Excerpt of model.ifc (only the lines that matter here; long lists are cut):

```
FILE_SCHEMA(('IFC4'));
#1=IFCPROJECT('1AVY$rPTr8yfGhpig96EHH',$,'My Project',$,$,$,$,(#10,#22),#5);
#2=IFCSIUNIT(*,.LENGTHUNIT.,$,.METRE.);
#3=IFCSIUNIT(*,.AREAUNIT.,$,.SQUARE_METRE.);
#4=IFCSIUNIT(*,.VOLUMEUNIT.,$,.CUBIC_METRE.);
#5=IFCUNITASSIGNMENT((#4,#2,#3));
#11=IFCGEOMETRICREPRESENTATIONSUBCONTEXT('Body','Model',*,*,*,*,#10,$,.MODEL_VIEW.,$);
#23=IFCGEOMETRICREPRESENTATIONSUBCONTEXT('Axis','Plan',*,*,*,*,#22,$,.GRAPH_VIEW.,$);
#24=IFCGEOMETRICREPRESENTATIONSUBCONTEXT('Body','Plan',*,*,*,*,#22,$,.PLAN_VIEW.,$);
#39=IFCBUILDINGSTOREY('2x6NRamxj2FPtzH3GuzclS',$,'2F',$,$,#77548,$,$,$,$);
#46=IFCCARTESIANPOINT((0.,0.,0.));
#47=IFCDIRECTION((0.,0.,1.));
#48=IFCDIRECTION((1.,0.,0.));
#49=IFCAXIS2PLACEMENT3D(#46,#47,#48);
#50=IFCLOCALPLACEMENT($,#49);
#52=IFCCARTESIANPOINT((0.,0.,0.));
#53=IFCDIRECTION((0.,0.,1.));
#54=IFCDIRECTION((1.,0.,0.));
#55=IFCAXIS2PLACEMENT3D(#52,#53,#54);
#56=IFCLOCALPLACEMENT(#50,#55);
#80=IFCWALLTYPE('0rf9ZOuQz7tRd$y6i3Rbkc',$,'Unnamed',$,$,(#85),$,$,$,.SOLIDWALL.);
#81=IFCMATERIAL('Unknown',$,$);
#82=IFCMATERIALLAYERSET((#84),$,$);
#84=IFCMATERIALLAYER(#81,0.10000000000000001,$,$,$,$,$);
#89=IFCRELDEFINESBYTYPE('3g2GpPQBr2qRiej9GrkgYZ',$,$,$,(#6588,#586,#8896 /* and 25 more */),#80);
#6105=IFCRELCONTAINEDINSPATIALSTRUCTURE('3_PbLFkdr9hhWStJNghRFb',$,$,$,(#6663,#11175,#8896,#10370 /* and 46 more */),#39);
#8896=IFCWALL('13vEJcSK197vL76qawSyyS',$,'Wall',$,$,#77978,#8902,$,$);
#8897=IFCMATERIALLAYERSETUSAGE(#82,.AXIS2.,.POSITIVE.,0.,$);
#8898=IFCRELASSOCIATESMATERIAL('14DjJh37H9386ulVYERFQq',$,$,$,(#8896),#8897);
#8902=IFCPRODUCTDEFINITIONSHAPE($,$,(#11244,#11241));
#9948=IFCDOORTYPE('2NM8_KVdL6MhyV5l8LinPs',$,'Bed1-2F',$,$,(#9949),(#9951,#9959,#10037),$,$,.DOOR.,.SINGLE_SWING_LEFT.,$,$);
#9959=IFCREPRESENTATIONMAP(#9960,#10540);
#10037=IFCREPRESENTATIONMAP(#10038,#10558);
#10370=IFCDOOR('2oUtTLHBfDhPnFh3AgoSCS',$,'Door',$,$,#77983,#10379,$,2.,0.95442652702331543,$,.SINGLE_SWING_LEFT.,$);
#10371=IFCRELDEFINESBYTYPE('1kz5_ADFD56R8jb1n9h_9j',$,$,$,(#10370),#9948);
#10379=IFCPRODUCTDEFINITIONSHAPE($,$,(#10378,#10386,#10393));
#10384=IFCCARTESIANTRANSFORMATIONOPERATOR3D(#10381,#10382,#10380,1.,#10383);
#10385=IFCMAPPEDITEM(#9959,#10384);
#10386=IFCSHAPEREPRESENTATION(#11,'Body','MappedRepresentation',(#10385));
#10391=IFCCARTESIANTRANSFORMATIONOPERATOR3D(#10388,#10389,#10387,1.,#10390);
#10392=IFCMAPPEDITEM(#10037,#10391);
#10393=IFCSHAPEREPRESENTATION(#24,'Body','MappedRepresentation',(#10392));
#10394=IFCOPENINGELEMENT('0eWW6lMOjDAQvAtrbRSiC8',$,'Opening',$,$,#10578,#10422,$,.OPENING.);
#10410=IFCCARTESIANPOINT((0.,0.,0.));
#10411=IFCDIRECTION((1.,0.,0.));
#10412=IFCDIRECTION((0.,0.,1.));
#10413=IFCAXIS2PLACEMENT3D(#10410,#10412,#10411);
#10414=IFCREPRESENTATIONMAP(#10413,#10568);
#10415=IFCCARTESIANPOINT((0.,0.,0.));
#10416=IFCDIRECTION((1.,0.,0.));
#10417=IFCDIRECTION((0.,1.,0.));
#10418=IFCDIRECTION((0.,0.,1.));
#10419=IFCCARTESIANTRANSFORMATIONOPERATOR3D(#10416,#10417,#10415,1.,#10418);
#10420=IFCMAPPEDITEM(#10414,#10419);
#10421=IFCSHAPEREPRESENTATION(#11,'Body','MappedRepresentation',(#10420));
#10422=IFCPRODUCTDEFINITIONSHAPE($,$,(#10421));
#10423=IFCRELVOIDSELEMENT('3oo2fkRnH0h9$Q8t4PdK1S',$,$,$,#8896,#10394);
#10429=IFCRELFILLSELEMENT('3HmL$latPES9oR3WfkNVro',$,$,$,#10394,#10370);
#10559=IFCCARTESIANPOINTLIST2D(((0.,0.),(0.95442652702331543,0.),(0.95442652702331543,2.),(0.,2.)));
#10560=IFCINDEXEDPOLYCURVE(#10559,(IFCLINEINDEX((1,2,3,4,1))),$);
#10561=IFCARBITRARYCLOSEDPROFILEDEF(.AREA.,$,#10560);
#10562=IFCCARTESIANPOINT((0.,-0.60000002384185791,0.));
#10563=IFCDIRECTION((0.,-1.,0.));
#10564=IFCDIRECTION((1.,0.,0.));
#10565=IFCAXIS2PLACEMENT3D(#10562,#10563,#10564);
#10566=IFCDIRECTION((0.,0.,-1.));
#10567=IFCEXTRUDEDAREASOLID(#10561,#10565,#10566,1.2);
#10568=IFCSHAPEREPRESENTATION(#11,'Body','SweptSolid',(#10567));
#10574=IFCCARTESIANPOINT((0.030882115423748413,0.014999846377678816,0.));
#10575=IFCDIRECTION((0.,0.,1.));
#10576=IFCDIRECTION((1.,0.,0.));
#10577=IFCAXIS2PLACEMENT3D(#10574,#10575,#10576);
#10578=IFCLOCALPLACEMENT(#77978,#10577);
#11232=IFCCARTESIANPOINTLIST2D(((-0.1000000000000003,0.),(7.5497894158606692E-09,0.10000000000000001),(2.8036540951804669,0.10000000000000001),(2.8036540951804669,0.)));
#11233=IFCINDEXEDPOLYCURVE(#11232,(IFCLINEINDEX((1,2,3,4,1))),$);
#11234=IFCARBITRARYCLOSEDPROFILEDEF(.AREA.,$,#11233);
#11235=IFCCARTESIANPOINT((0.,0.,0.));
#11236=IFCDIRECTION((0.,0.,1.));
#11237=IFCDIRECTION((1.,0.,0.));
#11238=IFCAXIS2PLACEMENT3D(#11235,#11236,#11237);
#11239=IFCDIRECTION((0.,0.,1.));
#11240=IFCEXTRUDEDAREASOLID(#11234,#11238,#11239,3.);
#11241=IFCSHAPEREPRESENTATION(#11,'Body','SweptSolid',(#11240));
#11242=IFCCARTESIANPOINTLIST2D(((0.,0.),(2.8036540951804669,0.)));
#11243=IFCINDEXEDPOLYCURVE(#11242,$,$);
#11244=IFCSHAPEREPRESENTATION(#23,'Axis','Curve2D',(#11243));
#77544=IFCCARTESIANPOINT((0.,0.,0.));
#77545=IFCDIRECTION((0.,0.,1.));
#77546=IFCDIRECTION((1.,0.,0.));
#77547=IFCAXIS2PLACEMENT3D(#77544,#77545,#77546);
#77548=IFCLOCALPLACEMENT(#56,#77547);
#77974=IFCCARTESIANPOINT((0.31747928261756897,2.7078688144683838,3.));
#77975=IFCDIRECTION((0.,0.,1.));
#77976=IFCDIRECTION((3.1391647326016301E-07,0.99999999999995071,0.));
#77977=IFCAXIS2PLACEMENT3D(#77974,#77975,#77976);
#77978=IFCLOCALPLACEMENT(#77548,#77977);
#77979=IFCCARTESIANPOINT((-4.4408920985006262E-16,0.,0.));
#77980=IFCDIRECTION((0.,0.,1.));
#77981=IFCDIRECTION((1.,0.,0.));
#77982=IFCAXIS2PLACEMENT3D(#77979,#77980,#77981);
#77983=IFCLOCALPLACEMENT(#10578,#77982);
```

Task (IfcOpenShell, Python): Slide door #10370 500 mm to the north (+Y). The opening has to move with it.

```python
import ifcopenshell
import ifcopenshell.api.geometry
import ifcopenshell.util.placement
import ifcopenshell.util.unit

model = ifcopenshell.open("model.ifc")
unit_scale = ifcopenshell.util.unit.calculate_unit_scale(model)

door = model.by_guid("2oUtTLHBfDhPnFh3AgoSCS")
opening = door.FillsVoids[0].RelatingOpeningElement
wall = opening.VoidsElements[0].RelatingBuildingElement

wall_matrix = ifcopenshell.util.placement.get_local_placement(wall.ObjectPlacement)
shift = wall_matrix[:3, 0] * 0.5 / unit_scale
before = ifcopenshell.util.placement.get_local_placement(door.ObjectPlacement)[:3, 3].copy()

# The door is placed relative to its opening, so it follows when the opening moves.
matrix = ifcopenshell.util.placement.get_local_placement(opening.ObjectPlacement)
matrix[:3, 3] += shift
ifcopenshell.api.geometry.edit_object_placement(
    model, product=opening, matrix=matrix, is_si=False, should_transform_children=True
)

after = ifcopenshell.util.placement.get_local_placement(door.ObjectPlacement)[:3, 3]
print("door moved by", (after - before).round(3) + 0.0)

model.write("model_edited.ifc")
```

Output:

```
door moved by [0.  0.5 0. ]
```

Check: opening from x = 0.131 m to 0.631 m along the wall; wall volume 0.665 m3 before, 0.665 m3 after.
